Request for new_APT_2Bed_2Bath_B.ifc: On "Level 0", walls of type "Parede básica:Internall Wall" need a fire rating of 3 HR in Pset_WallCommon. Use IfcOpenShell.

First a look at what the model holds.

```python
import ifcopenshell
import ifcopenshell.util.element

model = ifcopenshell.open("new_APT_2Bed_2Bath_B.ifc")
print(model.schema)
storey = next(s for s in model.by_type("IfcBuildingStorey") if s.Name == "Level 0")
walls = [e for e in ifcopenshell.util.element.get_decomposition(storey) if e.is_a("IfcWall")]
seen = {}
for e in walls:
    element_type = ifcopenshell.util.element.get_type(e)
    key = (element_type.Name if element_type != e and element_type else None, ifcopenshell.util.element.get_pset(e, "Pset_WallCommon", "FireRating"))
    seen[key] = seen.get(key, 0) + 1
for (name, value), count in sorted(seen.items(), key=str):
    print(count, "x", name, "|", value)
```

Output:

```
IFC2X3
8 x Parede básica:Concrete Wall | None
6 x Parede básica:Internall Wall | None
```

```python
import ifcopenshell
import ifcopenshell.api.pset
import ifcopenshell.util.element

model = ifcopenshell.open("new_APT_2Bed_2Bath_B.ifc")

storey = next(s for s in model.by_type("IfcBuildingStorey") if s.Name == "Level 0")
walls = [e for e in ifcopenshell.util.element.get_decomposition(storey) if e.is_a("IfcWall")]

count = 0
for e in walls:
    element_type = ifcopenshell.util.element.get_type(e)
    if element_type in (None, e) or element_type.Name != "Parede básica:Internall Wall":
        continue
    # add_pset returns the element's existing set when there is one.
    pset = ifcopenshell.api.pset.add_pset(model, product=e, name="Pset_WallCommon")
    ifcopenshell.api.pset.edit_pset(model, pset=pset, properties={"FireRating": "3 HR"})
    count += 1

print(count, "walls updated")

model.write("new_APT_2Bed_2Bath_B-out.ifc")
```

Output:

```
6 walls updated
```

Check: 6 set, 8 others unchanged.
